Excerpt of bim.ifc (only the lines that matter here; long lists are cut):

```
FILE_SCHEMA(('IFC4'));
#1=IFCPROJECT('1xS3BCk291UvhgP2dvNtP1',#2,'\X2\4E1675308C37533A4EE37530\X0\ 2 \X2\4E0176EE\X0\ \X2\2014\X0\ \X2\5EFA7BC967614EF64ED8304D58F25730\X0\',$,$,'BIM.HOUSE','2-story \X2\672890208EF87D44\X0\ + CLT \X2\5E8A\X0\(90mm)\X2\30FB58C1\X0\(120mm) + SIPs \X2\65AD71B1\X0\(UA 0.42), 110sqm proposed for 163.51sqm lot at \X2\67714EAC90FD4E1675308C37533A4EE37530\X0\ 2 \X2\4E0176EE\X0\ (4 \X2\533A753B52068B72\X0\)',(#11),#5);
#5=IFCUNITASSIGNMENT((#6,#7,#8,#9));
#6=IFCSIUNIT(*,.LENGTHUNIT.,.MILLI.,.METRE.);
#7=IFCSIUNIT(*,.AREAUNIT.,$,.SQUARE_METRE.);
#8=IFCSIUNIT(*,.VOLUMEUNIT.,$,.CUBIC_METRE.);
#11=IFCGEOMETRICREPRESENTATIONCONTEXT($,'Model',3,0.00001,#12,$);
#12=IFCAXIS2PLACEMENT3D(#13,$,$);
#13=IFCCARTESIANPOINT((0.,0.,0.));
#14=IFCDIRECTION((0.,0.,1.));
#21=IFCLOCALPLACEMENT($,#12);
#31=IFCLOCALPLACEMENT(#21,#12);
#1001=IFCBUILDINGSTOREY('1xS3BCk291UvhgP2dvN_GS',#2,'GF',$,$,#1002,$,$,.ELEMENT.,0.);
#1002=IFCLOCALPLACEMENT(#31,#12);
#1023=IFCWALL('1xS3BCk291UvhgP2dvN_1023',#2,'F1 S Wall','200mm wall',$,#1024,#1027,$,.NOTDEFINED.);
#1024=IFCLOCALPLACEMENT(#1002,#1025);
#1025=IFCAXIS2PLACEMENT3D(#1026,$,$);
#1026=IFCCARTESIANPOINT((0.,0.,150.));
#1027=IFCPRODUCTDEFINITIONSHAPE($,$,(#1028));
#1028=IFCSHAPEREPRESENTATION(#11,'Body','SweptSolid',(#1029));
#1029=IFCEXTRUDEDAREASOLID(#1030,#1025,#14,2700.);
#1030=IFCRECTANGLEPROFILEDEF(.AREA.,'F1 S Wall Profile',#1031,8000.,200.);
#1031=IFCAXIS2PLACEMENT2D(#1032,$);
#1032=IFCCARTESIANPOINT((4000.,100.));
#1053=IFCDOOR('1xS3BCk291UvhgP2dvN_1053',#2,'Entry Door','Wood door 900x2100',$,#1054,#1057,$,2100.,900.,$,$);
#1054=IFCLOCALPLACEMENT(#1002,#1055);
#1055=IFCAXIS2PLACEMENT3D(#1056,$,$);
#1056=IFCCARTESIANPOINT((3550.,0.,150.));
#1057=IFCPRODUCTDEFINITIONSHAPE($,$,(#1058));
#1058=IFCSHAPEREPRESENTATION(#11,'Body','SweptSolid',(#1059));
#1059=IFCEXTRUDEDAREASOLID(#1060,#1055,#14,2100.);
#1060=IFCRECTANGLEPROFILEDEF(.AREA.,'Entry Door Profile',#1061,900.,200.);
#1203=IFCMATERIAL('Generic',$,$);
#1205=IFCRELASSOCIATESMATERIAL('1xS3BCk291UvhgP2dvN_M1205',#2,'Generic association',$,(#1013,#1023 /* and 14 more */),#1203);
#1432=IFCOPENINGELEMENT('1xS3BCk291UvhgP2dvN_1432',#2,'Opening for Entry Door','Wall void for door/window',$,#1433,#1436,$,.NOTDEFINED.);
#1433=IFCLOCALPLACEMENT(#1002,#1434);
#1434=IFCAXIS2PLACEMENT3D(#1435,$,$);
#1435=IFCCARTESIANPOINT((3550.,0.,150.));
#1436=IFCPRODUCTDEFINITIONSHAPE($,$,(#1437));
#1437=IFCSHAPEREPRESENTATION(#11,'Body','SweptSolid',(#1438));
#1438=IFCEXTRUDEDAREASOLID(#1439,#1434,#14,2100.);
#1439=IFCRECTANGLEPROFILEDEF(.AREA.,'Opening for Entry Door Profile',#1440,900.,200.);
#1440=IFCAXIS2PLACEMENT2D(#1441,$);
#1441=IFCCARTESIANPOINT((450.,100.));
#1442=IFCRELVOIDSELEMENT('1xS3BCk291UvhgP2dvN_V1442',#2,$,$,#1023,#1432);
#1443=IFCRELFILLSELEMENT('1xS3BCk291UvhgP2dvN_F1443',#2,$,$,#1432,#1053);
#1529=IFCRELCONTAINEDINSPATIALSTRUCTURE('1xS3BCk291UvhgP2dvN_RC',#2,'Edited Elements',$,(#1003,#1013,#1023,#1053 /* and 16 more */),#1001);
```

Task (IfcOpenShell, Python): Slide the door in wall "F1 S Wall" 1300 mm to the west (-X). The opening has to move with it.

```python
import ifcopenshell
import ifcopenshell.api.geometry
import ifcopenshell.util.placement
import ifcopenshell.util.unit

model = ifcopenshell.open("bim.ifc")
unit_scale = ifcopenshell.util.unit.calculate_unit_scale(model)

door = model.by_guid("1xS3BCk291UvhgP2dvN_1053")
opening = door.FillsVoids[0].RelatingOpeningElement
wall = opening.VoidsElements[0].RelatingBuildingElement

wall_matrix = ifcopenshell.util.placement.get_local_placement(wall.ObjectPlacement)
shift = wall_matrix[:3, 0] * -1.3 / unit_scale
before = ifcopenshell.util.placement.get_local_placement(door.ObjectPlacement)[:3, 3].copy()

# The door is not placed relative to its opening, so move both.
for product in (opening, door):
    matrix = ifcopenshell.util.placement.get_local_placement(product.ObjectPlacement)
    matrix[:3, 3] += shift
    ifcopenshell.api.geometry.edit_object_placement(model, product=product, matrix=matrix, is_si=False)

after = ifcopenshell.util.placement.get_local_placement(door.ObjectPlacement)[:3, 3]
print("door moved by", (after - before).round(3) + 0.0)

model.write("bim_updated.ifc")
```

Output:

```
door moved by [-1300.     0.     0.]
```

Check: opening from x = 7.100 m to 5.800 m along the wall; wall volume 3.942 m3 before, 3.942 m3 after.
